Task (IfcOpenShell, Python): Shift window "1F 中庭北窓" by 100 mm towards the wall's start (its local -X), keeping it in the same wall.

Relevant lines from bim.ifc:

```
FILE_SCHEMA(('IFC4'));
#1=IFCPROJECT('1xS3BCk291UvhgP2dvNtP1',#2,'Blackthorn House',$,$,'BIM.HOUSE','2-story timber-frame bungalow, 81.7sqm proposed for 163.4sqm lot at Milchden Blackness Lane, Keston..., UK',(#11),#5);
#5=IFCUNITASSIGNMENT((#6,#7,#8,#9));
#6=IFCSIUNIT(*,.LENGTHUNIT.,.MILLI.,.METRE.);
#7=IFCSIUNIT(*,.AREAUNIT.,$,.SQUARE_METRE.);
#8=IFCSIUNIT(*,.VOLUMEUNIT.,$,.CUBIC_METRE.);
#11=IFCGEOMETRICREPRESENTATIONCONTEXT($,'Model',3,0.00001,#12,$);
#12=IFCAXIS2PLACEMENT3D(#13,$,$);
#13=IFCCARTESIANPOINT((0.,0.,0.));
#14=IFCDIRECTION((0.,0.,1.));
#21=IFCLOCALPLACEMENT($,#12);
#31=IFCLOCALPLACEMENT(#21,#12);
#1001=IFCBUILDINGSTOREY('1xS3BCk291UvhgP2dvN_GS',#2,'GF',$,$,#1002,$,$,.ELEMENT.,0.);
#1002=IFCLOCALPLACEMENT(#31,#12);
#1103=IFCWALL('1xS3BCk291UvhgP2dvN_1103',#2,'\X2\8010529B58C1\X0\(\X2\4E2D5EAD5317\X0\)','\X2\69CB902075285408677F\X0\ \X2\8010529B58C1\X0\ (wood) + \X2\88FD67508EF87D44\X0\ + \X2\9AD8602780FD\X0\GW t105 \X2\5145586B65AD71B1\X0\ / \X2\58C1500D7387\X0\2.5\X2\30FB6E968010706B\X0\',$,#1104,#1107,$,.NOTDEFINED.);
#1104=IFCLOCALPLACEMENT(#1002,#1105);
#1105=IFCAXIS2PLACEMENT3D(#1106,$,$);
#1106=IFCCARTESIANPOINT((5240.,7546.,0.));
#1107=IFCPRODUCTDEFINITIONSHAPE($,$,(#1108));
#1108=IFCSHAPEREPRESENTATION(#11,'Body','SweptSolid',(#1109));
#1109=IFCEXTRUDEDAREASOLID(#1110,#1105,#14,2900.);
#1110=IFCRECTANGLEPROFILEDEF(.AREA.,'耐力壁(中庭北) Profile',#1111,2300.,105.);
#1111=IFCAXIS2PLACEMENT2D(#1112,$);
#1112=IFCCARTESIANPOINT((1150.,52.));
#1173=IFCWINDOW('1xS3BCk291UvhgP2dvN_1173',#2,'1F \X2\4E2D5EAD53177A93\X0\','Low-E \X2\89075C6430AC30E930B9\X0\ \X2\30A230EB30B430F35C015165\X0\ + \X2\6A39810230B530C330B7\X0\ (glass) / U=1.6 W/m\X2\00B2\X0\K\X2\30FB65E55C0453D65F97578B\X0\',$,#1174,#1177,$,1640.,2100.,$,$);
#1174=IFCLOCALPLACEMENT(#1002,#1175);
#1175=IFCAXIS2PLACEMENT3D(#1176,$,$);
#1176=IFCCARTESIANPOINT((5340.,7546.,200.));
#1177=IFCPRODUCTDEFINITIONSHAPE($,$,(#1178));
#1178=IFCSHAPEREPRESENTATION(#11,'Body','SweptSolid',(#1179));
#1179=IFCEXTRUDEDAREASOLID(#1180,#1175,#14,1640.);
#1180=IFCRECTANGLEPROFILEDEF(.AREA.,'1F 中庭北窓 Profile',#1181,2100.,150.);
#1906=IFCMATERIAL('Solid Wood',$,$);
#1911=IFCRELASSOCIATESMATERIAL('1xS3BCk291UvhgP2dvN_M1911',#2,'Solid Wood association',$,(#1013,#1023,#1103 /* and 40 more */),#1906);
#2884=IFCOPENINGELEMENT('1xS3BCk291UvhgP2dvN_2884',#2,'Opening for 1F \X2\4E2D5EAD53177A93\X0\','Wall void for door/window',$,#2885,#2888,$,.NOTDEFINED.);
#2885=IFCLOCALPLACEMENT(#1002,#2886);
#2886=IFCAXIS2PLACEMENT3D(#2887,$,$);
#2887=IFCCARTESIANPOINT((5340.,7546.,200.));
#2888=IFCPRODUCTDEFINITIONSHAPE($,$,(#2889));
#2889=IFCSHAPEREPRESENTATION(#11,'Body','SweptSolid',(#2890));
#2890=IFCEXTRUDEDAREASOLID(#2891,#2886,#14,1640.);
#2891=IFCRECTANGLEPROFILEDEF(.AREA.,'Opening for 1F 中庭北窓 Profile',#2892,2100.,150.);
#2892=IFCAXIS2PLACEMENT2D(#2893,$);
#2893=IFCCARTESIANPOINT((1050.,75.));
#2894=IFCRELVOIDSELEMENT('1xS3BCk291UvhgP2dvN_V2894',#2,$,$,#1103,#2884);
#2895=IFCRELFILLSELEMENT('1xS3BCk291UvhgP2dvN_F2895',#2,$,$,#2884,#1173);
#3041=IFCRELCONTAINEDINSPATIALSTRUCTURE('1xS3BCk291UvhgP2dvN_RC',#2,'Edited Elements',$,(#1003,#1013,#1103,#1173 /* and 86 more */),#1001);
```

```python
import ifcopenshell
import ifcopenshell.api.geometry
import ifcopenshell.util.placement
import ifcopenshell.util.unit

model = ifcopenshell.open("bim.ifc")
unit_scale = ifcopenshell.util.unit.calculate_unit_scale(model)

window = model.by_guid("1xS3BCk291UvhgP2dvN_1173")
opening = window.FillsVoids[0].RelatingOpeningElement
wall = opening.VoidsElements[0].RelatingBuildingElement

wall_matrix = ifcopenshell.util.placement.get_local_placement(wall.ObjectPlacement)
shift = wall_matrix[:3, 0] * -0.1 / unit_scale
before = ifcopenshell.util.placement.get_local_placement(window.ObjectPlacement)[:3, 3].copy()

# The window is not placed relative to its opening, so move both.
for product in (opening, window):
    matrix = ifcopenshell.util.placement.get_local_placement(product.ObjectPlacement)
    matrix[:3, 3] += shift
    ifcopenshell.api.geometry.edit_object_placement(model, product=product, matrix=matrix, is_si=False)

after = ifcopenshell.util.placement.get_local_placement(window.ObjectPlacement)[:3, 3]
print("window moved by", (after - before).round(3) + 0.0)

model.write("bim_updated.ifc")
```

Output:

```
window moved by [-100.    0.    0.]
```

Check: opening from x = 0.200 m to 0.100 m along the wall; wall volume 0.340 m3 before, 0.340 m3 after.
